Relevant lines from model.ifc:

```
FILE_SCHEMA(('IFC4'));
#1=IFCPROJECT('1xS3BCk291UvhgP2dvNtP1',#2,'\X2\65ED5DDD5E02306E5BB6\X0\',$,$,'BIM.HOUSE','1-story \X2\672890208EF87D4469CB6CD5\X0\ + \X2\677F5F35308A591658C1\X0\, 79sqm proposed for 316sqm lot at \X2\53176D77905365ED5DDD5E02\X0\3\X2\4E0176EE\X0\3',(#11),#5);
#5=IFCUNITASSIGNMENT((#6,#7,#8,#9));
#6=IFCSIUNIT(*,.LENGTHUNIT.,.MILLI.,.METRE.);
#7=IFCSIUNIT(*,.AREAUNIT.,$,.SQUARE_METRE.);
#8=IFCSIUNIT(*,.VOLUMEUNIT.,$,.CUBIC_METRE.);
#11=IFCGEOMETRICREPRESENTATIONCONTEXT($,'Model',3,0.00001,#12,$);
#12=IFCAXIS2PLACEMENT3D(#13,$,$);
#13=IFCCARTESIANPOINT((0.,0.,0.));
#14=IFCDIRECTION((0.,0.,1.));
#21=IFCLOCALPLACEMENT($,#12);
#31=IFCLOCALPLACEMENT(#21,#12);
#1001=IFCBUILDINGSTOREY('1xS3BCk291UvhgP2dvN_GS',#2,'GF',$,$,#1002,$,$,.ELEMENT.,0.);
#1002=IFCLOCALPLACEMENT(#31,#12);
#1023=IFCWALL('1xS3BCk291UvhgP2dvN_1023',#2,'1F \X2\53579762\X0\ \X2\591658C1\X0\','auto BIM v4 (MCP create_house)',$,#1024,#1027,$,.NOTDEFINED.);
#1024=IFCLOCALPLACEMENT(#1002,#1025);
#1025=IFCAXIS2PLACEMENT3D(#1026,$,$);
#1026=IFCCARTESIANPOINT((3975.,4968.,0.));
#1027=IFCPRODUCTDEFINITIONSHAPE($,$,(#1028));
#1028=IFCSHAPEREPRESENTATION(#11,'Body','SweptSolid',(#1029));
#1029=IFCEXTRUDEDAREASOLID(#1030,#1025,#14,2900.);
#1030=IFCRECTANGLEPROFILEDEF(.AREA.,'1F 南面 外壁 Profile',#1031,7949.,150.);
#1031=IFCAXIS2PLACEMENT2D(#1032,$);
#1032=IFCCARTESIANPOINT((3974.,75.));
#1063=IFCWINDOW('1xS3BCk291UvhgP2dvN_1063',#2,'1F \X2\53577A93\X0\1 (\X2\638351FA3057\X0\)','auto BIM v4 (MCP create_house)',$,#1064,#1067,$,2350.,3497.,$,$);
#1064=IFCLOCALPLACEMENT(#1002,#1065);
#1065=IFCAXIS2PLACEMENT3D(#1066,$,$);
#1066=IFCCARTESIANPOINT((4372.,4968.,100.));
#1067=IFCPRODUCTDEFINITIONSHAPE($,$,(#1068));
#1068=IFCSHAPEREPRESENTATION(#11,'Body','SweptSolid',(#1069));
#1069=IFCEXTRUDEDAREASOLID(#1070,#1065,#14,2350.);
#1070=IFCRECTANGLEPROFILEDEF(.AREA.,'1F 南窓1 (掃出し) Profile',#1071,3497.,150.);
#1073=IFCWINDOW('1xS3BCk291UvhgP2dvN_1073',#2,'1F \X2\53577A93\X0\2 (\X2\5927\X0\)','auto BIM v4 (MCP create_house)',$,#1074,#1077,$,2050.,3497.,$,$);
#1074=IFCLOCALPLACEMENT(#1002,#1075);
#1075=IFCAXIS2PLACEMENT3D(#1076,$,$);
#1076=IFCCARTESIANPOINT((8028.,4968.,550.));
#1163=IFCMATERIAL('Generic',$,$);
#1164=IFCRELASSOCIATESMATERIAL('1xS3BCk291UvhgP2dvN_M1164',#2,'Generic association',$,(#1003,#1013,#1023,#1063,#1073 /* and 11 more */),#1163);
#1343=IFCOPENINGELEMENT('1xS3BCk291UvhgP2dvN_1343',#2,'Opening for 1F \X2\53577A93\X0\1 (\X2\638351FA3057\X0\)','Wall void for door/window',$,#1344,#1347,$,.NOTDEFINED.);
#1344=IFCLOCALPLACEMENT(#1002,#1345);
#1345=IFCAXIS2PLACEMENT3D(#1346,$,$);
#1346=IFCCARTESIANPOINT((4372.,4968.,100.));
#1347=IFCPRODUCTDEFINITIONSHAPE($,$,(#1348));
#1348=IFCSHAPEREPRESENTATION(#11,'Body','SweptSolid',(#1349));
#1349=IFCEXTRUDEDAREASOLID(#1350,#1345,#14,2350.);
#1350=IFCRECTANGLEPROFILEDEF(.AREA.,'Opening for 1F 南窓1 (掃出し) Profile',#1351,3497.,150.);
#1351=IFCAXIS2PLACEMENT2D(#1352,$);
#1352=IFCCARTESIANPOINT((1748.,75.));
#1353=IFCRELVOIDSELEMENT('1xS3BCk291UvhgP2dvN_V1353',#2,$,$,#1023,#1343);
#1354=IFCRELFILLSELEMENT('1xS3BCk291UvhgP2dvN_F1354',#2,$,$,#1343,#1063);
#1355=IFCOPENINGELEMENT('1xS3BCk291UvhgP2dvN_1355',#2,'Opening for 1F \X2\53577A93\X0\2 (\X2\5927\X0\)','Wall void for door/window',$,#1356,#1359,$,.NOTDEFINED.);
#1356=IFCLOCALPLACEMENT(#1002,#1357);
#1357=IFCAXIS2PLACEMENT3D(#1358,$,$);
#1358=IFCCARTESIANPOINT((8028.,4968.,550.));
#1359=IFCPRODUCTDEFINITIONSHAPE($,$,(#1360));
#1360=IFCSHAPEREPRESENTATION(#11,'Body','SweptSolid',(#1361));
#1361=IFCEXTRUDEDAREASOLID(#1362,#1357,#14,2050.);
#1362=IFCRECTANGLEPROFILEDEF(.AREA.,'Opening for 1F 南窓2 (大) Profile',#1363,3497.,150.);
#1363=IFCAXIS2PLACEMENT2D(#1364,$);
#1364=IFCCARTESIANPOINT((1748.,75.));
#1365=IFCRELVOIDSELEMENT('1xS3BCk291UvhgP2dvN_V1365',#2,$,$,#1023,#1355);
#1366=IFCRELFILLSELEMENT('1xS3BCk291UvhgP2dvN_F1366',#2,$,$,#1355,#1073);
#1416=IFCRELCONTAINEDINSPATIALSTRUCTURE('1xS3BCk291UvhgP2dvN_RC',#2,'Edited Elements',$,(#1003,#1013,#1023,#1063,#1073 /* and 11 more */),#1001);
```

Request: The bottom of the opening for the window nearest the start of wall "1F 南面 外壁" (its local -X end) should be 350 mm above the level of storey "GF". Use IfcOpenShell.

```python
import numpy as np
import ifcopenshell
import ifcopenshell.api.geometry
import ifcopenshell.geom
import ifcopenshell.util.element
import ifcopenshell.util.placement
import ifcopenshell.util.shape
import ifcopenshell.util.unit

model = ifcopenshell.open("model.ifc")
unit_scale = ifcopenshell.util.unit.calculate_unit_scale(model)

window = model.by_guid("1xS3BCk291UvhgP2dvN_1063")
opening = window.FillsVoids[0].RelatingOpeningElement
storey = ifcopenshell.util.element.get_container(window, ifc_class="IfcBuildingStorey")
level = ifcopenshell.util.placement.get_local_placement(storey.ObjectPlacement)[2, 3]

# The opening's origin need not be at the sill, so measure its lowest point.
shape = ifcopenshell.geom.create_shape(ifcopenshell.geom.settings(), opening)
bottom = ifcopenshell.util.shape.get_shape_bottom_elevation(shape, shape.geometry) / unit_scale
dz = level + 350.0 - bottom

shift = np.array([0.0, 0.0, dz])
# The window is not placed relative to its opening, so move both.
for product in (opening, window):
    matrix = ifcopenshell.util.placement.get_local_placement(product.ObjectPlacement)
    matrix[:3, 3] += shift
    ifcopenshell.api.geometry.edit_object_placement(model, product=product, matrix=matrix, is_si=False)

print(f"moved by {dz * unit_scale:+.3f} m")

model.write("model-out.ifc")
```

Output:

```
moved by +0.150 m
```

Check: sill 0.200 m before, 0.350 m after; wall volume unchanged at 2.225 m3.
